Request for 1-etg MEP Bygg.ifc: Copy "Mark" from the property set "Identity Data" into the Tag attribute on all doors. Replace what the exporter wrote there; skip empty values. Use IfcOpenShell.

First a look at what the model holds.

```python
import ifcopenshell
import ifcopenshell.util.element

model = ifcopenshell.open("1-etg MEP Bygg.ifc")
print(model.schema)
doors = model.by_type("IfcDoor")
print(len(doors), "doors")
for e in doors[:8]:
    source = ifcopenshell.util.element.get_pset(e, "Identity Data", "Mark")
    target = e.Tag
    print(e.id(), repr(source), repr(target), sep=" | ")
```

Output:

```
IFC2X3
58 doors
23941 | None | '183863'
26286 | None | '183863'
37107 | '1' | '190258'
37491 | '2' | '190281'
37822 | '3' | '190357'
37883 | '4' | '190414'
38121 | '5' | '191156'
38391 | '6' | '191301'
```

```python
import ifcopenshell
import ifcopenshell.util.element

model = ifcopenshell.open("1-etg MEP Bygg.ifc")

count = 0
for e in model.by_type("IfcDoor"):
    value = ifcopenshell.util.element.get_pset(e, "Identity Data", "Mark")
    current = e.Tag
    if not value or not value.strip() or current == value:
        continue
    e.Tag = value
    count += 1

print(count, "doors updated")

model.write("1-etg MEP Bygg-out.ifc")
```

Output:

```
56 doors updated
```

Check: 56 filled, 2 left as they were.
